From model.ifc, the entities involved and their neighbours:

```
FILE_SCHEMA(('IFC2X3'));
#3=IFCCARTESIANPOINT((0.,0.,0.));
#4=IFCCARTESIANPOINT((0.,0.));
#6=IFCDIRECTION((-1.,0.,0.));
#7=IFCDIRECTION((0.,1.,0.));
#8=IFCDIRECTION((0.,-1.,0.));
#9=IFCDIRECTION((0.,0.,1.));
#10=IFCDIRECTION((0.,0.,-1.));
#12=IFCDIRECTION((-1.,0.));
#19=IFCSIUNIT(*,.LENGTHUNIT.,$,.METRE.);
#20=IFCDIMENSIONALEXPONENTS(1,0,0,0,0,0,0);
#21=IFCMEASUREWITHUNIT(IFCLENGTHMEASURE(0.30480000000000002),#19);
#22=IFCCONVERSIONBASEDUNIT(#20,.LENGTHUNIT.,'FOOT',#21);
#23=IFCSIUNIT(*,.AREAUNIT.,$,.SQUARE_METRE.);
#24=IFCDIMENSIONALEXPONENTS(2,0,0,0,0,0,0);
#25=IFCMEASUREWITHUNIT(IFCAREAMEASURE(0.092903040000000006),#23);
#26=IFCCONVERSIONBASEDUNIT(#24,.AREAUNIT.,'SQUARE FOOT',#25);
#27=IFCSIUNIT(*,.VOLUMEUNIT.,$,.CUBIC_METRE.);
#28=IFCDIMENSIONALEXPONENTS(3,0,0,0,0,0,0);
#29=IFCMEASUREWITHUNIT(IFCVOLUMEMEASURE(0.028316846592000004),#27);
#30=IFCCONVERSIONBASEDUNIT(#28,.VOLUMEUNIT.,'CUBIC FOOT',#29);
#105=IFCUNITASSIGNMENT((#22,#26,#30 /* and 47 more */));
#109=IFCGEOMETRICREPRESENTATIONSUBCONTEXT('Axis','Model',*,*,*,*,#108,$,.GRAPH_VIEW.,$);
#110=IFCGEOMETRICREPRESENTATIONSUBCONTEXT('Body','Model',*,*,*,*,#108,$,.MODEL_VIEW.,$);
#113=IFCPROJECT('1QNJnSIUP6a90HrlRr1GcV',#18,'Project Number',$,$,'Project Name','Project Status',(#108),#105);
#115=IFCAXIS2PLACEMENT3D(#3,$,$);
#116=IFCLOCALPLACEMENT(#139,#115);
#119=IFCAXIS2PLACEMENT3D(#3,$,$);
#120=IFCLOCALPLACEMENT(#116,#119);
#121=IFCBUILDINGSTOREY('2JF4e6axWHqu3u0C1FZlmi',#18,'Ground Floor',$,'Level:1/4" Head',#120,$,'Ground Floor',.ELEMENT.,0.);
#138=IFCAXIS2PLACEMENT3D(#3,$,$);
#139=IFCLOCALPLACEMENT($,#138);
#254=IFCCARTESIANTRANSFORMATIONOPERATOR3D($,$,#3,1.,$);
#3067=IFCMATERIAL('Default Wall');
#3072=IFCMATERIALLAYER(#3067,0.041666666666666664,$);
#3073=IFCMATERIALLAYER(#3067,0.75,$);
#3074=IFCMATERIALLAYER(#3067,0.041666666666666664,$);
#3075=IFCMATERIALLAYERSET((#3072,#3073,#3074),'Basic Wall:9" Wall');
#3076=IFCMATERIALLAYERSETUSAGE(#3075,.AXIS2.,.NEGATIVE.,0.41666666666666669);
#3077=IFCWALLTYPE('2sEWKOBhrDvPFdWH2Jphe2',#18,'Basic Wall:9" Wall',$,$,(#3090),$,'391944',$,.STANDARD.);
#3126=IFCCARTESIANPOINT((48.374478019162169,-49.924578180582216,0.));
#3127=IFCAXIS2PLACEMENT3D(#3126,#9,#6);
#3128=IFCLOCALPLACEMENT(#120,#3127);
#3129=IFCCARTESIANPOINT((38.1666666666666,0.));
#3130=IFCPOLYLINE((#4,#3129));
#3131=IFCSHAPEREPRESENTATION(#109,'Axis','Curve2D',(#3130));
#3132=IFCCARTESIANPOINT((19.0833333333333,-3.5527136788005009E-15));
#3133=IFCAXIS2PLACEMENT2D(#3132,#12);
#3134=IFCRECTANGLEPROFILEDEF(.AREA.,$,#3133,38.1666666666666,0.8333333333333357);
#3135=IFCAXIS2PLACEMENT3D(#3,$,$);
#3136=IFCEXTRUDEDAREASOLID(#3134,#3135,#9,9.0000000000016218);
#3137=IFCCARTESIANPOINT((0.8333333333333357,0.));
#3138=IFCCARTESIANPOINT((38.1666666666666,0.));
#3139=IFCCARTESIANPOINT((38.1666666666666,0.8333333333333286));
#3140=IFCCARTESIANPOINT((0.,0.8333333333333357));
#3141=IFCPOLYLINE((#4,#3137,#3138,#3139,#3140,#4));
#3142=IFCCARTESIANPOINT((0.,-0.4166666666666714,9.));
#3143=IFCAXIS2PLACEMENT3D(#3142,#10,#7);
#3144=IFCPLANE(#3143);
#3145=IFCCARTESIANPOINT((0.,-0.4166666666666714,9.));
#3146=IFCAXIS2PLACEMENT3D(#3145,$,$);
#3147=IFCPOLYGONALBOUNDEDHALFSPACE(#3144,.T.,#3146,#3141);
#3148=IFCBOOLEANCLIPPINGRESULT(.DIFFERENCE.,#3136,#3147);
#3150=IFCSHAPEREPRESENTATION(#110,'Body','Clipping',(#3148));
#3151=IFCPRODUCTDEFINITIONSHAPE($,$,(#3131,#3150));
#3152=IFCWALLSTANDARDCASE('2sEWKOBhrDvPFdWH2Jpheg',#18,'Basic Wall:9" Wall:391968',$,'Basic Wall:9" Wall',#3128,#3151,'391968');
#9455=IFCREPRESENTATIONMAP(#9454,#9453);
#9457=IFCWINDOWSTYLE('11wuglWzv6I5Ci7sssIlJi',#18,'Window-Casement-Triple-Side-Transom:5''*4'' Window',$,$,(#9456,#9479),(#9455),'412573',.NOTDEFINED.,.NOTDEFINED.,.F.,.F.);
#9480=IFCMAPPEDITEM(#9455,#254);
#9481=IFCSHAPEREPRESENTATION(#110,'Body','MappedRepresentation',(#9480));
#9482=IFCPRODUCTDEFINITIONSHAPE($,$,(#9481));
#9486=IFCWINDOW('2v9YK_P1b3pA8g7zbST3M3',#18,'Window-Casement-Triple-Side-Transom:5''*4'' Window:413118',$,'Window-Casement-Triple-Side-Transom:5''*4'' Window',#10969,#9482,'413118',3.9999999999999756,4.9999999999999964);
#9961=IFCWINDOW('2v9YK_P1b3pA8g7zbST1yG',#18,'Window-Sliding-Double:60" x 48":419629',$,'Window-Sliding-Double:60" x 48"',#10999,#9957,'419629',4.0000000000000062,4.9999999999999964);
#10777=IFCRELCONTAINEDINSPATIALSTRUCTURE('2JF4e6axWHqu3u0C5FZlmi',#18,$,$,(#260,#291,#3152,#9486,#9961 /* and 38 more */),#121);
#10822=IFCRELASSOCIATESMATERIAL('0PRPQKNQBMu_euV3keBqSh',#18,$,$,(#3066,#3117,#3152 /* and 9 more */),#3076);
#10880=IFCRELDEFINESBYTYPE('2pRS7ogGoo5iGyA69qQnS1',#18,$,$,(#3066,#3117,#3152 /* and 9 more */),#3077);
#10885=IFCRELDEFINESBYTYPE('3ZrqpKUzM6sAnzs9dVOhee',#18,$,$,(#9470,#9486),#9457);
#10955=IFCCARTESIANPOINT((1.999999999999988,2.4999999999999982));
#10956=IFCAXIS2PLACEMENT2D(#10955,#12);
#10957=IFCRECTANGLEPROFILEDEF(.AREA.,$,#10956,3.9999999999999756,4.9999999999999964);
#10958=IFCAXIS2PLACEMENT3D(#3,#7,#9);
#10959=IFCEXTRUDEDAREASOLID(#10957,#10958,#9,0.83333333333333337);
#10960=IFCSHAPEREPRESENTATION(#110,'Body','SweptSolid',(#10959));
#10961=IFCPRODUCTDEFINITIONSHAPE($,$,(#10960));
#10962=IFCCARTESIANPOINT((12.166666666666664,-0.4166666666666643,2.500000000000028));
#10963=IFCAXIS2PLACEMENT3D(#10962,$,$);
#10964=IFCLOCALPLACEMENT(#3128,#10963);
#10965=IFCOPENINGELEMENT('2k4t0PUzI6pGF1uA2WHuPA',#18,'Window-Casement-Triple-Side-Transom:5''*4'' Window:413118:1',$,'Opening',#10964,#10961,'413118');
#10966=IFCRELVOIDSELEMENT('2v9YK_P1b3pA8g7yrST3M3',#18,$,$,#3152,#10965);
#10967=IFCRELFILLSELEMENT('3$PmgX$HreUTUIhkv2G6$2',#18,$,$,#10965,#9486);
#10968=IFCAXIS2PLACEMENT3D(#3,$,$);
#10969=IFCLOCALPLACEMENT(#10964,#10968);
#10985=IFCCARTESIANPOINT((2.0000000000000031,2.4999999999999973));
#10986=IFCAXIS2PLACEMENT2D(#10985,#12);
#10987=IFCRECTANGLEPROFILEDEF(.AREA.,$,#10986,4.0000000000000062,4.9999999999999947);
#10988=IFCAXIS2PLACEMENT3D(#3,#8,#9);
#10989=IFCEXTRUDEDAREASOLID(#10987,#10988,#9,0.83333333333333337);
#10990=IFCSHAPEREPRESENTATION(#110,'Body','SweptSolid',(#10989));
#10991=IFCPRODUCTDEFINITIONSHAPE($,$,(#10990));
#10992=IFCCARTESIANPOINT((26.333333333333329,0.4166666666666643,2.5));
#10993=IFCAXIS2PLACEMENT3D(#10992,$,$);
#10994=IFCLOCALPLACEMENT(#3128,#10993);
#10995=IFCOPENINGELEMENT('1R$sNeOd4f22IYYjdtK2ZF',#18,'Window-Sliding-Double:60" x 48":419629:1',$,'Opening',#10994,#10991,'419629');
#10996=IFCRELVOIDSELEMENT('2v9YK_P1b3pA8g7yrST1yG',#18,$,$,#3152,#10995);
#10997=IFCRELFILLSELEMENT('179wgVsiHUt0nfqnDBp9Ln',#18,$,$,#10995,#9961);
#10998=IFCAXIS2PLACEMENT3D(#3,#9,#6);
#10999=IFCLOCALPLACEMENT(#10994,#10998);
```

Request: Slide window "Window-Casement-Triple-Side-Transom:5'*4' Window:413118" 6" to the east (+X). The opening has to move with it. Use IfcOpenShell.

```python
import ifcopenshell
import ifcopenshell.api.geometry
import ifcopenshell.util.placement
import ifcopenshell.util.unit

model = ifcopenshell.open("model.ifc")
unit_scale = ifcopenshell.util.unit.calculate_unit_scale(model)

window = model.by_guid("2v9YK_P1b3pA8g7zbST3M3")
opening = window.FillsVoids[0].RelatingOpeningElement
wall = opening.VoidsElements[0].RelatingBuildingElement

wall_matrix = ifcopenshell.util.placement.get_local_placement(wall.ObjectPlacement)
shift = wall_matrix[:3, 0] * -6 * 0.0254 / unit_scale
before = ifcopenshell.util.placement.get_local_placement(window.ObjectPlacement)[:3, 3].copy()

# The window is placed relative to its opening, so it follows when the opening moves.
matrix = ifcopenshell.util.placement.get_local_placement(opening.ObjectPlacement)
matrix[:3, 3] += shift
ifcopenshell.api.geometry.edit_object_placement(
    model, product=opening, matrix=matrix, is_si=False, should_transform_children=True
)

after = ifcopenshell.util.placement.get_local_placement(window.ObjectPlacement)[:3, 3]
print("window moved by", (after - before).round(3) + 0.0)

model.write("model-out.ifc")
```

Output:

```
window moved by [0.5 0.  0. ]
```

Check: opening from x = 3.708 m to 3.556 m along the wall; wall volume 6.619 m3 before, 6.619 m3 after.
